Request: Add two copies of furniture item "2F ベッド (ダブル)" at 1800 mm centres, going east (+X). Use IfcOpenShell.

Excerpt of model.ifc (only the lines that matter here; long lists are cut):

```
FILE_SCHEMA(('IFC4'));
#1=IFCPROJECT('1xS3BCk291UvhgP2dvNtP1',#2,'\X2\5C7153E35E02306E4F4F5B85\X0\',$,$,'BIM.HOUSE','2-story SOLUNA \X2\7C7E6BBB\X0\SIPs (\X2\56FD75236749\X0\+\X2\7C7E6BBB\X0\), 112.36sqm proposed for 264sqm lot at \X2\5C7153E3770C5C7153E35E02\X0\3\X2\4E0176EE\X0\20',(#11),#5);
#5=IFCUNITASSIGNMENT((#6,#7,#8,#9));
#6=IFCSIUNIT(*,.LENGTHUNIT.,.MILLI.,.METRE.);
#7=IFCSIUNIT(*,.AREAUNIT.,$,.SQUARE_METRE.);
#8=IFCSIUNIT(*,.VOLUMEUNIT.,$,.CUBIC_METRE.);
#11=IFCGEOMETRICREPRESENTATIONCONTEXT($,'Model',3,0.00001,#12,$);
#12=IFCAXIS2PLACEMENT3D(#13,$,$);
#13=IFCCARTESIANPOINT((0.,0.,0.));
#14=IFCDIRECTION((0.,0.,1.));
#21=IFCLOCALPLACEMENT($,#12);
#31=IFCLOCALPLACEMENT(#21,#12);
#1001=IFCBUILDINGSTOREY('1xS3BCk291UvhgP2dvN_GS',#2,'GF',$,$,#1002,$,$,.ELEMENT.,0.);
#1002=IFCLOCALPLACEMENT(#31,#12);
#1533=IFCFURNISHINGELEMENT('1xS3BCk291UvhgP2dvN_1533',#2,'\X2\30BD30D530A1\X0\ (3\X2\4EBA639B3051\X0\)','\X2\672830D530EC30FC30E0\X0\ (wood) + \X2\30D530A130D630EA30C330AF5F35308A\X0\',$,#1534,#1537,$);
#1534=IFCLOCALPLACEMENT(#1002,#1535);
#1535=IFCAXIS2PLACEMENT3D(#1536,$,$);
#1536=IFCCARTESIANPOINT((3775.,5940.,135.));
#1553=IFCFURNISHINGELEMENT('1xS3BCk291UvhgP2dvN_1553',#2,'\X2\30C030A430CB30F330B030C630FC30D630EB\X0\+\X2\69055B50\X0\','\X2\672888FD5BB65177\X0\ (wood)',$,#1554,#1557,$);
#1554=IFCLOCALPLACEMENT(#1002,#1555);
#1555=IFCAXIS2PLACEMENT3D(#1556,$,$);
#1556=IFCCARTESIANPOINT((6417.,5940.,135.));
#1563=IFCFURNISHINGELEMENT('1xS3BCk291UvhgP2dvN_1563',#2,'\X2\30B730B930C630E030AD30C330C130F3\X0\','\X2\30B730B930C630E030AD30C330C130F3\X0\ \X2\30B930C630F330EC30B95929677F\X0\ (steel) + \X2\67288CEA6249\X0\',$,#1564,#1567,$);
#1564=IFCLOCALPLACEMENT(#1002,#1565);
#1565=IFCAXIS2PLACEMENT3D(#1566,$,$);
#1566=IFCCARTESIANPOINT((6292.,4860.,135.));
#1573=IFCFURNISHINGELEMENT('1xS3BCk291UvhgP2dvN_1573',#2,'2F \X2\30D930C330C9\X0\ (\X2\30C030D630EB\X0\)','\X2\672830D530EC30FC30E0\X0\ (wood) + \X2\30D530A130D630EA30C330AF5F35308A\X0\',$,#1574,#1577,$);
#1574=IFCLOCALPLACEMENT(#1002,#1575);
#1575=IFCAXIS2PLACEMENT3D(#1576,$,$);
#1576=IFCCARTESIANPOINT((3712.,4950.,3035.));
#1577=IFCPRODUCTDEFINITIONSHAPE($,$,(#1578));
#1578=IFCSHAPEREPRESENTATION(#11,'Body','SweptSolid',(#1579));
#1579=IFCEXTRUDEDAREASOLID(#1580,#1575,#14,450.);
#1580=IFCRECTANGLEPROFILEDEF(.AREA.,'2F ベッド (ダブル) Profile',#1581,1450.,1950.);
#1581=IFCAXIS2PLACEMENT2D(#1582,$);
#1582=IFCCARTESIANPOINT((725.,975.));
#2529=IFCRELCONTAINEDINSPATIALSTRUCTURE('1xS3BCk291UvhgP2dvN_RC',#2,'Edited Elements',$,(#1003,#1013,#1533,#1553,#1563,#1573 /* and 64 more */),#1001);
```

```python
import numpy as np
import ifcopenshell
import ifcopenshell.api.geometry
import ifcopenshell.api.root
import ifcopenshell.util.element
import ifcopenshell.util.placement
import ifcopenshell.util.unit

model = ifcopenshell.open("model.ifc")
unit_scale = ifcopenshell.util.unit.calculate_unit_scale(model)


def reuse_history(source, copy):
    """copy_class also copies each property set's owner history, people and application; keep the originals."""
    for rel in copy.IsDefinedBy:
        if rel.is_a("IfcRelDefinesByProperties") and (history := rel.RelatingPropertyDefinition.OwnerHistory):
            rel.RelatingPropertyDefinition.OwnerHistory = source.OwnerHistory
            ifcopenshell.util.element.remove_deep2(model, history)


source = model.by_id(1573)
base = ifcopenshell.util.placement.get_local_placement(source.ObjectPlacement)
step = np.array([1.0, 0.0, 0.0]) * 1.8 / unit_scale

for i in range(1, 3):
    copy = ifcopenshell.api.root.copy_class(model, product=source)
    copy.Representation = ifcopenshell.util.element.copy_deep(
        model, source.Representation, exclude=["IfcGeometricRepresentationContext", "IfcRepresentationMap"]
    )
    reuse_history(source, copy)
    matrix = base.copy()
    matrix[:3, 3] += i * step
    print("added at", matrix[:3, 3].round(3) + 0.0)
    ifcopenshell.api.geometry.edit_object_placement(model, product=copy, matrix=matrix, is_si=False)

model.write("model_rev.ifc")
```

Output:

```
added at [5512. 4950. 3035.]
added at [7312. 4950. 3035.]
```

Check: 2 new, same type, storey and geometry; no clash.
